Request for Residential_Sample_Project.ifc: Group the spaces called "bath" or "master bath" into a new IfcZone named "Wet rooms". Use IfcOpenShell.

First a look at what the model holds.

```python
import ifcopenshell

model = ifcopenshell.open("Residential_Sample_Project.ifc")
print(model.schema)
seen = {}
for space in model.by_type("IfcSpace"):
    seen[space.LongName] = seen.get(space.LongName, 0) + 1
for name, count in sorted(seen.items(), key=str):
    print(count, "x", name)
print("zones:", [z.Name for z in model.by_type("IfcZone")][:20])
```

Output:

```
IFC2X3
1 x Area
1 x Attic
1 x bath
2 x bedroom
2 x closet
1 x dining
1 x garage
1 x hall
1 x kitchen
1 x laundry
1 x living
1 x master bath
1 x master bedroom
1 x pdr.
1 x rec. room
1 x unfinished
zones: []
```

```python
import ifcopenshell
import ifcopenshell.api.group
import ifcopenshell.api.root

model = ifcopenshell.open("Residential_Sample_Project.ifc")

names = {"bath", "master bath"}
spaces = [s for s in model.by_type("IfcSpace") if s.LongName in names]

zone = ifcopenshell.api.root.create_entity(model, ifc_class="IfcZone", name="Wet rooms")
ifcopenshell.api.group.assign_group(model, products=spaces, group=zone)
print(len(spaces), "spaces in", zone.Name)

model.write("Residential_Sample_Project_v2.ifc")
```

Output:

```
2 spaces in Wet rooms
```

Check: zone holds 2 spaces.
